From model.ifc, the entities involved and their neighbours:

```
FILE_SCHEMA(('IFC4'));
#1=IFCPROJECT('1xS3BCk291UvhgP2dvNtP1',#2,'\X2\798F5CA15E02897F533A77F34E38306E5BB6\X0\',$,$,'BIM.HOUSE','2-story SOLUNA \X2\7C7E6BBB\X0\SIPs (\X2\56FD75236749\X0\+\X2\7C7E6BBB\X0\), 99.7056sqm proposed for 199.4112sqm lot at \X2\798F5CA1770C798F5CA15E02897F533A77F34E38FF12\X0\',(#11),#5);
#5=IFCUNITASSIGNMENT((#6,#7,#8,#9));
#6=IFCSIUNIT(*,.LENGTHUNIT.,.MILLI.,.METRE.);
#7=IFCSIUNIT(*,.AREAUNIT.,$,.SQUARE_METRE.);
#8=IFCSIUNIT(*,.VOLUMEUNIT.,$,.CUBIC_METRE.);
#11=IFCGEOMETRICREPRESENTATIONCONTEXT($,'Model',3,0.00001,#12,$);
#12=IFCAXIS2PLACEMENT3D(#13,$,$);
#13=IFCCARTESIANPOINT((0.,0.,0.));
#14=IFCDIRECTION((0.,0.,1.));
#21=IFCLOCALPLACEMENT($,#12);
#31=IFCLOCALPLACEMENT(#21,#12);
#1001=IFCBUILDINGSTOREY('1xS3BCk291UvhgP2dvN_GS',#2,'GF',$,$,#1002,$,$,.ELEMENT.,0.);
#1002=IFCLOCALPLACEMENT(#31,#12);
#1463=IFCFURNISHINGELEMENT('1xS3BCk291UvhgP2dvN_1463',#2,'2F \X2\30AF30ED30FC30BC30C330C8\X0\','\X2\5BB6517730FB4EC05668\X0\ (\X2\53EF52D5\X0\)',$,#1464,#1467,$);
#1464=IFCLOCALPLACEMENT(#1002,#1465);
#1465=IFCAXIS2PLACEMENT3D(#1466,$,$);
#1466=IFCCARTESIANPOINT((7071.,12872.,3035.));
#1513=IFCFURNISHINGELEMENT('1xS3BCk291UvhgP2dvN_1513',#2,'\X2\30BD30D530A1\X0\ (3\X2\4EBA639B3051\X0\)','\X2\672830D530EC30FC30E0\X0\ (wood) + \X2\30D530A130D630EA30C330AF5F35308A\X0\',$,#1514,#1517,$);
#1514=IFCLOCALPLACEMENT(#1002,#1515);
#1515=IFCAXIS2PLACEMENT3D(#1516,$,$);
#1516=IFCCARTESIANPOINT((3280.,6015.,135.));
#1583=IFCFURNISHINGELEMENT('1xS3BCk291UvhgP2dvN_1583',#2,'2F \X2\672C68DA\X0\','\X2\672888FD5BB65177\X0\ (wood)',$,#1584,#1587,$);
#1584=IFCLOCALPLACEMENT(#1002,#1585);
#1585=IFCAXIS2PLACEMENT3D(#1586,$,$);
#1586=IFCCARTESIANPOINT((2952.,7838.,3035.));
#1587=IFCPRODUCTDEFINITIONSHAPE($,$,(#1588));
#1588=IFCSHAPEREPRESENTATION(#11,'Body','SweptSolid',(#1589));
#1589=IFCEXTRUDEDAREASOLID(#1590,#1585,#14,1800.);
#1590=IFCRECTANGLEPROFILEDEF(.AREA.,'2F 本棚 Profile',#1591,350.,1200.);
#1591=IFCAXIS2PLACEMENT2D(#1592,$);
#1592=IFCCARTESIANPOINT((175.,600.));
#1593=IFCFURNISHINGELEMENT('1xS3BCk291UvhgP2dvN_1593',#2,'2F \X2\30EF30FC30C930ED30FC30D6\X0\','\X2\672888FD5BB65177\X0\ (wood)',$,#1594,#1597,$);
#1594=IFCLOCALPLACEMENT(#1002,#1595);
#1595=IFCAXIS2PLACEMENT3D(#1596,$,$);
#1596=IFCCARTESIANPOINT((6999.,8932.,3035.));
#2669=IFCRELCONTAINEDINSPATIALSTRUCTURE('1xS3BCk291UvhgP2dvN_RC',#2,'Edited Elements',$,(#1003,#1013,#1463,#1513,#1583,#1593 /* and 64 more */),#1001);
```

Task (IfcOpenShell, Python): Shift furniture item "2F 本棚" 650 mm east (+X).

```python
import ifcopenshell
import ifcopenshell.api.geometry
import ifcopenshell.util.placement
import ifcopenshell.util.unit

model = ifcopenshell.open("model.ifc")
unit_scale = ifcopenshell.util.unit.calculate_unit_scale(model)

item = model.by_id(1583)
matrix = ifcopenshell.util.placement.get_local_placement(item.ObjectPlacement)
matrix[0, 3] += 0.65 / unit_scale
ifcopenshell.api.geometry.edit_object_placement(model, product=item, matrix=matrix, is_si=False)

print(ifcopenshell.util.placement.get_local_placement(item.ObjectPlacement).round(3) + 0.0)

model.write("model_edited.ifc")
```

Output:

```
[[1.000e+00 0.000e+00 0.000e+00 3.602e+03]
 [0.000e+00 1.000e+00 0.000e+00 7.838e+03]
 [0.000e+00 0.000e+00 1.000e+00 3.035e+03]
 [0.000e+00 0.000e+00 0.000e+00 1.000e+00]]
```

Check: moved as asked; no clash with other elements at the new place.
